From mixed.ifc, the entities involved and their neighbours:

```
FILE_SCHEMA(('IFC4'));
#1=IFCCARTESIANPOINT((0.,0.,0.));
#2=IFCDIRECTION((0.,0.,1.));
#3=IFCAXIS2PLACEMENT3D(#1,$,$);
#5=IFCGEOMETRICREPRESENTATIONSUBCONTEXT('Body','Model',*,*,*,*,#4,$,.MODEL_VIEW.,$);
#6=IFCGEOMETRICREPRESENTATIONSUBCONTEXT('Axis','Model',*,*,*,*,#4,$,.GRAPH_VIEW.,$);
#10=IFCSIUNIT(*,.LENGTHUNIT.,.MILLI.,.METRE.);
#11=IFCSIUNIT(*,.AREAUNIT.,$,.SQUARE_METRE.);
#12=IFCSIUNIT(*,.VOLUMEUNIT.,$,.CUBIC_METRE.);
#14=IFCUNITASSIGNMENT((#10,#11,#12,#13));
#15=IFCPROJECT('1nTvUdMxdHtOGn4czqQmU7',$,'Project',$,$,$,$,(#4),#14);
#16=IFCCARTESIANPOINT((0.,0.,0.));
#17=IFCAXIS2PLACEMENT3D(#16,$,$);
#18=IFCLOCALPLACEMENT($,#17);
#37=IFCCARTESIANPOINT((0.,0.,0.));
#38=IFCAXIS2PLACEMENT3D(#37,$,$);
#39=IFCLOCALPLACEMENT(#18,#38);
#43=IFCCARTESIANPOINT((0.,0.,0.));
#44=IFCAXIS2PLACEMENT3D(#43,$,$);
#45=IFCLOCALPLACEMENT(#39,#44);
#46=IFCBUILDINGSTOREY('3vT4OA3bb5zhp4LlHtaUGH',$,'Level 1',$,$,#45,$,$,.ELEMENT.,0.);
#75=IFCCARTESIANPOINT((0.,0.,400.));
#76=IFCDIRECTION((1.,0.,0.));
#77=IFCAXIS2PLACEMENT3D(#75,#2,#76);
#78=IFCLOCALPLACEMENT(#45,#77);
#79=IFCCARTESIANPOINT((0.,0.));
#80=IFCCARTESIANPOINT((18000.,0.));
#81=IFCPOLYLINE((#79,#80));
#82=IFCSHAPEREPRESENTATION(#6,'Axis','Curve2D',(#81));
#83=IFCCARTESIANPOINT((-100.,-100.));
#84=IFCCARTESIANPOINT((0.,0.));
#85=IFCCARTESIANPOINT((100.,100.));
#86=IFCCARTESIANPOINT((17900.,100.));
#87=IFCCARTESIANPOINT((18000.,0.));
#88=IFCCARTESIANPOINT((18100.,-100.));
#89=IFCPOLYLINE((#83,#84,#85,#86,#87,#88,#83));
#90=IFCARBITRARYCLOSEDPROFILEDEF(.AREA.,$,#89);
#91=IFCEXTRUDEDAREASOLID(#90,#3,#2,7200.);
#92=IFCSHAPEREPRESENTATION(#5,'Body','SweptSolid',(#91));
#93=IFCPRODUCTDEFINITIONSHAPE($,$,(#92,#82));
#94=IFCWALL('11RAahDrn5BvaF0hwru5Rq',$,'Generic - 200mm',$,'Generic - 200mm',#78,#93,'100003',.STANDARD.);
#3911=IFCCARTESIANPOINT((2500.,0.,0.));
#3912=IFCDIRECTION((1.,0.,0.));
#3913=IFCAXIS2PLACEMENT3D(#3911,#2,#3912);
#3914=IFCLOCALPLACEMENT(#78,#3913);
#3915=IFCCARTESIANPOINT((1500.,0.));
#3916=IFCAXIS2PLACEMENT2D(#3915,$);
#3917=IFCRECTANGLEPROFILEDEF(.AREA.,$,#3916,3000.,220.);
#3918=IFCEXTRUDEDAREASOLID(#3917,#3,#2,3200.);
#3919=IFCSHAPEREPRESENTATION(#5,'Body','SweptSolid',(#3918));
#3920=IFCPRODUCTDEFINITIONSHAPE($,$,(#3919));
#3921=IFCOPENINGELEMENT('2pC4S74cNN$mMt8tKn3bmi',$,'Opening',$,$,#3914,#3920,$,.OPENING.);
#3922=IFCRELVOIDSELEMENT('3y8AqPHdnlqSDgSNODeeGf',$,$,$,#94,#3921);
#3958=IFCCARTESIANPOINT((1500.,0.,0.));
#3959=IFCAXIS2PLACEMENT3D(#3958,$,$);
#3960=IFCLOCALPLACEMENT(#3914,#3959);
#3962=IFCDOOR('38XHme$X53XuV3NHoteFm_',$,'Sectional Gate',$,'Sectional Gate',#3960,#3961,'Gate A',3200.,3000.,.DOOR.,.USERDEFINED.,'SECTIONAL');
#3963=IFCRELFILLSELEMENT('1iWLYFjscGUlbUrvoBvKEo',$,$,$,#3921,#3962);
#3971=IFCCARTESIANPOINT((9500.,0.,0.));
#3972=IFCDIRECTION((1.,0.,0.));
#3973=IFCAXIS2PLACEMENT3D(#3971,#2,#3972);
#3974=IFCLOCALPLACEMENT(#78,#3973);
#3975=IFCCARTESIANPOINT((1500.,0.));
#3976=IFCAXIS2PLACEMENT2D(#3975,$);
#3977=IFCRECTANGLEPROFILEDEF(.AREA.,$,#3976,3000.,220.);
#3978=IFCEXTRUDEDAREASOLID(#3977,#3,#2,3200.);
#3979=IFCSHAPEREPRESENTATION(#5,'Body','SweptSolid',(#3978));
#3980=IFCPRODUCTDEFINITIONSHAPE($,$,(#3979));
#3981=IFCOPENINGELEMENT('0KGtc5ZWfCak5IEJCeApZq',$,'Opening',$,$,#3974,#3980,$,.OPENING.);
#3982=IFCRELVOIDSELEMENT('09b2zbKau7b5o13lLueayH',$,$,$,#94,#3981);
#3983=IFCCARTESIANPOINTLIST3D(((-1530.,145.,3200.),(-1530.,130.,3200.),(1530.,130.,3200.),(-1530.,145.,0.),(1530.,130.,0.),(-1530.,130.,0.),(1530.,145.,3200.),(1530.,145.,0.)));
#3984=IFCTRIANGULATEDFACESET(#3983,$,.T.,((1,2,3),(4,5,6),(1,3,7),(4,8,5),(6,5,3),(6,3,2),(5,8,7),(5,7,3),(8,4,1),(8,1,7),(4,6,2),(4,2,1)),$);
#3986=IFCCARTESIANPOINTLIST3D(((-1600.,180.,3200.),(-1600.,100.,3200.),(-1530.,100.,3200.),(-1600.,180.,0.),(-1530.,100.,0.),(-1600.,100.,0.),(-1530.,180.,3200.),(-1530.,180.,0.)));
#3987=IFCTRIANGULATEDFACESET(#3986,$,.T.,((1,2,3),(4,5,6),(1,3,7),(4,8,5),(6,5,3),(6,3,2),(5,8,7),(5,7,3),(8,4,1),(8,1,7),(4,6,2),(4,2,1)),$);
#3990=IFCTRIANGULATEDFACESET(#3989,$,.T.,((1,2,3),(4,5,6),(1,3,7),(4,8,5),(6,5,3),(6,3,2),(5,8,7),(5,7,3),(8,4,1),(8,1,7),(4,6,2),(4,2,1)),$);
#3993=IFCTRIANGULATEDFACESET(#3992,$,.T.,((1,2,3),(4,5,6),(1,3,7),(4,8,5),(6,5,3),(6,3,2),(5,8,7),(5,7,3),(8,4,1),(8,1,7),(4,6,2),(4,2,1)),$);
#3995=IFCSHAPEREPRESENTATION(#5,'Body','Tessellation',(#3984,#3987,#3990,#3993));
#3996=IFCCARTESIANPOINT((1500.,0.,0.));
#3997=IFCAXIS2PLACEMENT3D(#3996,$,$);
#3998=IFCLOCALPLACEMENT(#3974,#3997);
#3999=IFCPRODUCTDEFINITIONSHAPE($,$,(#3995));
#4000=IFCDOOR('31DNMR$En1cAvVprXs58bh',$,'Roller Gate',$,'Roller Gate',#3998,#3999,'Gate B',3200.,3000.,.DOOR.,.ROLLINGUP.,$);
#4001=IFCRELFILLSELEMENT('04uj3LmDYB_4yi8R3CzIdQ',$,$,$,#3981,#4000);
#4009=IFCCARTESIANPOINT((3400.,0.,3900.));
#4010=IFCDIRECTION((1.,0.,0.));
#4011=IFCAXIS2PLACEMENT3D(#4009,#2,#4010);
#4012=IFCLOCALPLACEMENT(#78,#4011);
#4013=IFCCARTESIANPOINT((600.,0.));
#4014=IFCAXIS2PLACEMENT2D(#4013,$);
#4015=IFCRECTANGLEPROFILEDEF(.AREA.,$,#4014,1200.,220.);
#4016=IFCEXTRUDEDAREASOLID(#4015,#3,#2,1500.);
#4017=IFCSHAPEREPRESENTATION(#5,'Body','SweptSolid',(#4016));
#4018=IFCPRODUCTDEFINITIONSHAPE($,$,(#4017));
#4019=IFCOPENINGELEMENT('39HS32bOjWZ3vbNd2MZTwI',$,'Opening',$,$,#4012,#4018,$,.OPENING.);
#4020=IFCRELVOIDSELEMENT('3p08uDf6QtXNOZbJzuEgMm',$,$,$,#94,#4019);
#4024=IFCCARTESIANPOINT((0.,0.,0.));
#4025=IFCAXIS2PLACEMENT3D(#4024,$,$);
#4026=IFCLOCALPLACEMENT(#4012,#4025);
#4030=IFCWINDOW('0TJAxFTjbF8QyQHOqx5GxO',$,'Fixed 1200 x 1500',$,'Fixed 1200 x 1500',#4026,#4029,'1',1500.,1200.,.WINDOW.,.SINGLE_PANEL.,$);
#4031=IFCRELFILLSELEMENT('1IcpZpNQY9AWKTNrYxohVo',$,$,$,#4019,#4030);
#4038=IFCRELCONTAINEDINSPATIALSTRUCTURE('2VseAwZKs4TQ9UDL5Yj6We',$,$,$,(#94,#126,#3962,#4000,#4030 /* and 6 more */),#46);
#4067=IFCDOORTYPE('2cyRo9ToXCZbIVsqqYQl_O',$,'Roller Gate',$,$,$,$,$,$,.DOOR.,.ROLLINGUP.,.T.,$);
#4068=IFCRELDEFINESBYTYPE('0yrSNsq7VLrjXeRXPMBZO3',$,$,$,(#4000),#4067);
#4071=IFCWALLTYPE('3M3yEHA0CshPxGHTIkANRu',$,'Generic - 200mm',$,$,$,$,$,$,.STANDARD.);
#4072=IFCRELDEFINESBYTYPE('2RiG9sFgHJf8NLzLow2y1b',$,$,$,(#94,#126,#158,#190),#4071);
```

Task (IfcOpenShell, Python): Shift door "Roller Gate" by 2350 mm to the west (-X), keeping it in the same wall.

```python
import ifcopenshell
import ifcopenshell.api.geometry
import ifcopenshell.util.placement
import ifcopenshell.util.unit

model = ifcopenshell.open("mixed.ifc")
unit_scale = ifcopenshell.util.unit.calculate_unit_scale(model)

door = model.by_id(4000)
opening = door.FillsVoids[0].RelatingOpeningElement
wall = opening.VoidsElements[0].RelatingBuildingElement

wall_matrix = ifcopenshell.util.placement.get_local_placement(wall.ObjectPlacement)
shift = wall_matrix[:3, 0] * -2.35 / unit_scale
before = ifcopenshell.util.placement.get_local_placement(door.ObjectPlacement)[:3, 3].copy()

# The door is placed relative to its opening, so it follows when the opening moves.
matrix = ifcopenshell.util.placement.get_local_placement(opening.ObjectPlacement)
matrix[:3, 3] += shift
ifcopenshell.api.geometry.edit_object_placement(
    model, product=opening, matrix=matrix, is_si=False, should_transform_children=True
)

after = ifcopenshell.util.placement.get_local_placement(door.ObjectPlacement)[:3, 3]
print("door moved by", (after - before).round(3) + 0.0)

model.write("mixed_edited.ifc")
```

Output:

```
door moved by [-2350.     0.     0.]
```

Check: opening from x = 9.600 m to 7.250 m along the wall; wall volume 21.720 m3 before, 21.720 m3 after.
